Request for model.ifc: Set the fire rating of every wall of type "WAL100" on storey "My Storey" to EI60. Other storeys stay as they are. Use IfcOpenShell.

First a look at what the model holds.

```python
import ifcopenshell
import ifcopenshell.util.element

model = ifcopenshell.open("model.ifc")
print(model.schema)
storey = next(s for s in model.by_type("IfcBuildingStorey") if s.Name == "My Storey")
walls = [e for e in ifcopenshell.util.element.get_decomposition(storey) if e.is_a("IfcWall")]
seen = {}
for e in walls:
    element_type = ifcopenshell.util.element.get_type(e)
    key = (element_type.Name if element_type != e and element_type else None, ifcopenshell.util.element.get_pset(e, "Pset_WallCommon", "FireRating"))
    seen[key] = seen.get(key, 0) + 1
for (name, value), count in sorted(seen.items(), key=str):
    print(count, "x", name, "|", value)
```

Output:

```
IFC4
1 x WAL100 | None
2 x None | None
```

```python
import ifcopenshell
import ifcopenshell.api.pset
import ifcopenshell.util.element

model = ifcopenshell.open("model.ifc")

storey = next(s for s in model.by_type("IfcBuildingStorey") if s.Name == "My Storey")
walls = [e for e in ifcopenshell.util.element.get_decomposition(storey) if e.is_a("IfcWall")]

count = 0
for e in walls:
    element_type = ifcopenshell.util.element.get_type(e)
    if element_type in (None, e) or element_type.Name != "WAL100":
        continue
    # add_pset returns the element's existing set when there is one.
    pset = ifcopenshell.api.pset.add_pset(model, product=e, name="Pset_WallCommon")
    ifcopenshell.api.pset.edit_pset(model, pset=pset, properties={"FireRating": "EI60"})
    count += 1

print(count, "walls updated")

model.write("model_edited.ifc")
```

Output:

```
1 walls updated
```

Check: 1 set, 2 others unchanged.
